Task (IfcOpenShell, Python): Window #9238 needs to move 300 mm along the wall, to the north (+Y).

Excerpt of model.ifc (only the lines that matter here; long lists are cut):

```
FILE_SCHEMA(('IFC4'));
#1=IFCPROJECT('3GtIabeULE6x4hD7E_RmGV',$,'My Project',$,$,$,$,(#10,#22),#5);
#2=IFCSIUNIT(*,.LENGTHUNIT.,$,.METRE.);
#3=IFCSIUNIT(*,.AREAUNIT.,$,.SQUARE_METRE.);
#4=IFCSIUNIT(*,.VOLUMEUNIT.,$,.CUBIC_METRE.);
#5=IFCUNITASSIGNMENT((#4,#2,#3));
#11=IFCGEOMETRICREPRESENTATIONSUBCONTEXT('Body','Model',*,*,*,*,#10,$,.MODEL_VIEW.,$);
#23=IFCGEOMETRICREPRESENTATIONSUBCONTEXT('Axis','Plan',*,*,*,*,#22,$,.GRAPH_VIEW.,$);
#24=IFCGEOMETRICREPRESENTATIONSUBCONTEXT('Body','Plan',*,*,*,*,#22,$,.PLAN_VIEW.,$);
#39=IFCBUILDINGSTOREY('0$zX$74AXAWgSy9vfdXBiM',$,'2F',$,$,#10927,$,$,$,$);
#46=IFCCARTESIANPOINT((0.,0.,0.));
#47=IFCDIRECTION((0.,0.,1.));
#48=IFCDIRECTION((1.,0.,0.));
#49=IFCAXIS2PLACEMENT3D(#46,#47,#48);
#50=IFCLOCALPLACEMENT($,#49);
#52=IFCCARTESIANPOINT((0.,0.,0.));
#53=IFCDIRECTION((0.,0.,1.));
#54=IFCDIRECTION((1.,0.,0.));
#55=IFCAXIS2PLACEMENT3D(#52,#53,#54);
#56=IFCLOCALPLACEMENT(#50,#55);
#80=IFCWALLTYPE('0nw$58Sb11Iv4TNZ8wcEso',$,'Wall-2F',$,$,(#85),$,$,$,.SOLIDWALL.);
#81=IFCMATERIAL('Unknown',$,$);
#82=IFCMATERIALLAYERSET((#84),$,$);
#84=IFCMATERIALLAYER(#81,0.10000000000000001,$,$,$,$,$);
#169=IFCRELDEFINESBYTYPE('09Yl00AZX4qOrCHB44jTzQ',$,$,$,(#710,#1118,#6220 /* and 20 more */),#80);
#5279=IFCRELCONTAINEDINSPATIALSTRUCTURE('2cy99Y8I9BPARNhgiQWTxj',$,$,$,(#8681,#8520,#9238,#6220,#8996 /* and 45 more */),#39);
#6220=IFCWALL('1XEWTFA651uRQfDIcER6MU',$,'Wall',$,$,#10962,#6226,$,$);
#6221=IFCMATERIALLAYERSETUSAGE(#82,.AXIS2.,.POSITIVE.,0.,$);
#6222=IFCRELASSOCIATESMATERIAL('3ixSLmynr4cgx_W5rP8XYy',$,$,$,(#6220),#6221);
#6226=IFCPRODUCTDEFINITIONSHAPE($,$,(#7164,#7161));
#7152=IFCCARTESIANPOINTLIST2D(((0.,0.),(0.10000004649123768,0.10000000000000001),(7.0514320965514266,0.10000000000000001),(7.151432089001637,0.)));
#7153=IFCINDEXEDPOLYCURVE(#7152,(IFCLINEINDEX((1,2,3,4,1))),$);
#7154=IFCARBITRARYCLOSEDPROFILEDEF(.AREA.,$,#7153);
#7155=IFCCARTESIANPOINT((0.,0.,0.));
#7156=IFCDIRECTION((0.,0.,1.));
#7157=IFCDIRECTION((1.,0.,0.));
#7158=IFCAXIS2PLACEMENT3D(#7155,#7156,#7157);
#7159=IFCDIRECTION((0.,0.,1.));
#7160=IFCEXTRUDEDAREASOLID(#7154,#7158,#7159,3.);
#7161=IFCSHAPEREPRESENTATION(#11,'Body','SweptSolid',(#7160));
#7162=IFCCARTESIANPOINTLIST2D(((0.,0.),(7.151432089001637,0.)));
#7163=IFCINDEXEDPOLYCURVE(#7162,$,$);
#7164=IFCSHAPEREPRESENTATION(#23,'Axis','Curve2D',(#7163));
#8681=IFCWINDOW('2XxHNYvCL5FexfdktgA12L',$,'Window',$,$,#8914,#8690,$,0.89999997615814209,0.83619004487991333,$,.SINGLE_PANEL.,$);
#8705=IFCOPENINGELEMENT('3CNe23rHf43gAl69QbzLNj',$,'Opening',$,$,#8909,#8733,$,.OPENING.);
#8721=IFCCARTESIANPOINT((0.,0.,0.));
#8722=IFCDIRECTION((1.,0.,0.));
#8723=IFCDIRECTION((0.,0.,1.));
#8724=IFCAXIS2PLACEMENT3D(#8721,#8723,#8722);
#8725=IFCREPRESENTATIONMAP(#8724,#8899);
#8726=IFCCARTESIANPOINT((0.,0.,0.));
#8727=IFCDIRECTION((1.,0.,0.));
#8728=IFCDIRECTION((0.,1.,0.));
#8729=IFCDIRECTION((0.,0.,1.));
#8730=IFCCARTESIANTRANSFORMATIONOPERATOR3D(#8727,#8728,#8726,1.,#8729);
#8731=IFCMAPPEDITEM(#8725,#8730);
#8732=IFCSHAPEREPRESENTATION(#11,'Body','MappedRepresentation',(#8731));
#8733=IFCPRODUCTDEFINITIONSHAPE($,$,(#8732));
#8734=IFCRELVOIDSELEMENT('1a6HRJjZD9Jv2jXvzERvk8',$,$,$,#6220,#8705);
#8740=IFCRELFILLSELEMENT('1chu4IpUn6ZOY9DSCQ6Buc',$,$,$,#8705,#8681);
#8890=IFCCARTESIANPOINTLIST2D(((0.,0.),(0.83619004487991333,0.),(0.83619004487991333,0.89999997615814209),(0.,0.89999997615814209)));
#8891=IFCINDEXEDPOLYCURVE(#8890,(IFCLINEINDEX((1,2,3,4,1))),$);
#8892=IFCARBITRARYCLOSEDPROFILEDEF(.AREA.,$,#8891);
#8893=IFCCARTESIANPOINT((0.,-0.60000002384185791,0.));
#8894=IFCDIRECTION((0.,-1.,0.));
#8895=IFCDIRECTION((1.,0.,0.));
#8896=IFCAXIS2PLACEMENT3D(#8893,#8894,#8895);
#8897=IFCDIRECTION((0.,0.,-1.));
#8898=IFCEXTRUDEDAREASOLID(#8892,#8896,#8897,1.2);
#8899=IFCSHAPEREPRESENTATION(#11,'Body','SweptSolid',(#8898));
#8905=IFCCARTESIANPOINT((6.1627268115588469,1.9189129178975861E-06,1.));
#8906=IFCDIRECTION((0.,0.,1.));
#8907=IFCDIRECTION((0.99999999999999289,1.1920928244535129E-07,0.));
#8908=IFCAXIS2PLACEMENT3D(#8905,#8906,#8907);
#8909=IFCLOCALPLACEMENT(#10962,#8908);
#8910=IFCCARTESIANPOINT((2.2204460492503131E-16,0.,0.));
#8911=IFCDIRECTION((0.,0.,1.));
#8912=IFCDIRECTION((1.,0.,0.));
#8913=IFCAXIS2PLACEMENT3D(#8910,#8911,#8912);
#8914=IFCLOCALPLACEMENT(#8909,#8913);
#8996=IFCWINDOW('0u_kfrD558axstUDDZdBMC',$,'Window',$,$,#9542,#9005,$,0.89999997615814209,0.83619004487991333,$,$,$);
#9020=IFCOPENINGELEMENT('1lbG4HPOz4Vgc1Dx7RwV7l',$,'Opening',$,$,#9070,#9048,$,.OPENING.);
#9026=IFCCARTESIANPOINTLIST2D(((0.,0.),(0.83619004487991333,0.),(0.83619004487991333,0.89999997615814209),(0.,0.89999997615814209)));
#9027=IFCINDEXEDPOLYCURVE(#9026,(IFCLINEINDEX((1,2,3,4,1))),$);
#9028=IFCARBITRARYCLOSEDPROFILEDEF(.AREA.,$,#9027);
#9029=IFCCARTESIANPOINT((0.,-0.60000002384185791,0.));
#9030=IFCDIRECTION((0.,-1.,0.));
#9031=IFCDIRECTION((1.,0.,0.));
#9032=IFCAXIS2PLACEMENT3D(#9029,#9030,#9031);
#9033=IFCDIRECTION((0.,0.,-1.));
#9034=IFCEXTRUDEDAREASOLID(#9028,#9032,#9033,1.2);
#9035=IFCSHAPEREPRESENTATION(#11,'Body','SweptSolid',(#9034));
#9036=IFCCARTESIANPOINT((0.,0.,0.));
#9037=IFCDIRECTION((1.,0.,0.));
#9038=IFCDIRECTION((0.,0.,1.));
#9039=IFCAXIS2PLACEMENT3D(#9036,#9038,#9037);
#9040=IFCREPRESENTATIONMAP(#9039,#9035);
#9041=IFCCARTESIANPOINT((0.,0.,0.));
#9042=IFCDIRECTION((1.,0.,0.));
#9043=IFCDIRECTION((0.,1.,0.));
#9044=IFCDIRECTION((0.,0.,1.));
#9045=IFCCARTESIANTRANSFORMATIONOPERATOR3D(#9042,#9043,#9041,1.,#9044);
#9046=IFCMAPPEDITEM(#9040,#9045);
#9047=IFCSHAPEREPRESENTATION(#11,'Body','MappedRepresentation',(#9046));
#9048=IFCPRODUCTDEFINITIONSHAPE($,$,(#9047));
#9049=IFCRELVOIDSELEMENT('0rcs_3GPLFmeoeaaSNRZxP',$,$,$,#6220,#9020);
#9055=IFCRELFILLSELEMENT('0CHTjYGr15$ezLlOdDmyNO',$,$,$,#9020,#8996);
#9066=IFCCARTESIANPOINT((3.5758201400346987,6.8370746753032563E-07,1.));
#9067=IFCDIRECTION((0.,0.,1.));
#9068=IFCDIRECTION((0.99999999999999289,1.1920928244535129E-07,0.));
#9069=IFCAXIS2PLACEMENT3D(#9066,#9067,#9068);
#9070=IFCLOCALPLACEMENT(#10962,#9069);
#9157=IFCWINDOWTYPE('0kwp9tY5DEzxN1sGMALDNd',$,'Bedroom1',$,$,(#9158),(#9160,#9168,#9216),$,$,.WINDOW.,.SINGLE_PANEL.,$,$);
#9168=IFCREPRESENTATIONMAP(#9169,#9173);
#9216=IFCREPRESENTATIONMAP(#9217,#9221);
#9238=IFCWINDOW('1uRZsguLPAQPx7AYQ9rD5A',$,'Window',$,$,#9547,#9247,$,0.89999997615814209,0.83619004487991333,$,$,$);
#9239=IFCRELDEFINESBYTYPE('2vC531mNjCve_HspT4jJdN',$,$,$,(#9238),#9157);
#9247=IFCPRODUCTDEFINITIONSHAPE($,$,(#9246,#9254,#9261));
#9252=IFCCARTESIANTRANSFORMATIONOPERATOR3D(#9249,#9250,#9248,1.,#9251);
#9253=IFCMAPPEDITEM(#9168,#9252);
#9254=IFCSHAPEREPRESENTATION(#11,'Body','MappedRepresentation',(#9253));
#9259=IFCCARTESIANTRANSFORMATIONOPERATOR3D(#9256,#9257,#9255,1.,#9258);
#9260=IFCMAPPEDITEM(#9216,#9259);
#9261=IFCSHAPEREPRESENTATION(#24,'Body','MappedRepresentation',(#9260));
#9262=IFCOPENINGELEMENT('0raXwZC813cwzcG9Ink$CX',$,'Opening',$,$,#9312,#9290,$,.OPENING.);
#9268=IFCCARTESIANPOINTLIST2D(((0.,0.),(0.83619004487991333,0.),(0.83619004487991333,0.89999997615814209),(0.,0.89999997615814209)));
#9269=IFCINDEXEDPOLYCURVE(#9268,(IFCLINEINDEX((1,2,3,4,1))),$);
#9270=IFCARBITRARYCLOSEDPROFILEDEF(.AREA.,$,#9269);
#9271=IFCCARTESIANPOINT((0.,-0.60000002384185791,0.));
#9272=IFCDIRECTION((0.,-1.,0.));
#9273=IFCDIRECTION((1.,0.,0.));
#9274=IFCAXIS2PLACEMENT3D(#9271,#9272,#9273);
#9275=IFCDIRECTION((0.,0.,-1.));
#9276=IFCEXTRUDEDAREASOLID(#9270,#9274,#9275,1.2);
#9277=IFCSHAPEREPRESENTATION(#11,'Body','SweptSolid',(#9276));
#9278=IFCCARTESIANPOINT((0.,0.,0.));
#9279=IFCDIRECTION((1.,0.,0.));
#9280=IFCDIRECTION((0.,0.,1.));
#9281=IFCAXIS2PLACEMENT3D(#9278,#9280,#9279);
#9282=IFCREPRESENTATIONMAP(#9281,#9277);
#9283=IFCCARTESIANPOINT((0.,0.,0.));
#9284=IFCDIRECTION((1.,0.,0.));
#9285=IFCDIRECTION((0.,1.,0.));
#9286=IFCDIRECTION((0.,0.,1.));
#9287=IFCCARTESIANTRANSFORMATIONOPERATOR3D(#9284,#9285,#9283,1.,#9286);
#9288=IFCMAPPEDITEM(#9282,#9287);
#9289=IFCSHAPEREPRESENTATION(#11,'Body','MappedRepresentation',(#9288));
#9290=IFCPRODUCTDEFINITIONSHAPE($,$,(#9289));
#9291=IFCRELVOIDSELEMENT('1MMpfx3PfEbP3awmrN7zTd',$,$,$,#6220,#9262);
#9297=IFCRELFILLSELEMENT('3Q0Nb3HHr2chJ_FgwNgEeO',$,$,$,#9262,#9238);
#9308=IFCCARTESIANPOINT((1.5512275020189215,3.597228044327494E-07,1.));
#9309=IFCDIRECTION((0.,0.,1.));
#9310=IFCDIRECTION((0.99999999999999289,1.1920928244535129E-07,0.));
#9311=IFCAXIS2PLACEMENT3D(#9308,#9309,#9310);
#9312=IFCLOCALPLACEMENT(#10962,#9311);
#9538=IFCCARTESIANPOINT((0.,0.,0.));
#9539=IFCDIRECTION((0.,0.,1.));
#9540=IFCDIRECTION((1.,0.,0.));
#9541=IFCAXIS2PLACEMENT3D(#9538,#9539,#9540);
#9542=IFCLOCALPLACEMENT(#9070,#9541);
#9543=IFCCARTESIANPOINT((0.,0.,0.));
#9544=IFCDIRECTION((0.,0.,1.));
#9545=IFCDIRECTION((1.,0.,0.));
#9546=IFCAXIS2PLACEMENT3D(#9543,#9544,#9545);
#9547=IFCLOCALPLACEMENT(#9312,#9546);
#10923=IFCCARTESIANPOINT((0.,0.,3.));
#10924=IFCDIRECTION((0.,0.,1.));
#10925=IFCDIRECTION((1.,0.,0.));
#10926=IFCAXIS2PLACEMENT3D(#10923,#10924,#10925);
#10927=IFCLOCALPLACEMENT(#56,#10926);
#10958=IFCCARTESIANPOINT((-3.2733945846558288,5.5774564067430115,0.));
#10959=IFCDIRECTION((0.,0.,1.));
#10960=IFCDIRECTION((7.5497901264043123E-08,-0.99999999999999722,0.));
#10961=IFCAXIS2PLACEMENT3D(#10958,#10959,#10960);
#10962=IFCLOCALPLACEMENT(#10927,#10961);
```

```python
import ifcopenshell
import ifcopenshell.api.geometry
import ifcopenshell.util.placement
import ifcopenshell.util.unit

model = ifcopenshell.open("model.ifc")
unit_scale = ifcopenshell.util.unit.calculate_unit_scale(model)

window = model.by_guid("1uRZsguLPAQPx7AYQ9rD5A")
opening = window.FillsVoids[0].RelatingOpeningElement
wall = opening.VoidsElements[0].RelatingBuildingElement

wall_matrix = ifcopenshell.util.placement.get_local_placement(wall.ObjectPlacement)
shift = wall_matrix[:3, 0] * -0.3 / unit_scale
before = ifcopenshell.util.placement.get_local_placement(window.ObjectPlacement)[:3, 3].copy()

# The window is placed relative to its opening, so it follows when the opening moves.
matrix = ifcopenshell.util.placement.get_local_placement(opening.ObjectPlacement)
matrix[:3, 3] += shift
ifcopenshell.api.geometry.edit_object_placement(
    model, product=opening, matrix=matrix, is_si=False, should_transform_children=True
)

after = ifcopenshell.util.placement.get_local_placement(window.ObjectPlacement)[:3, 3]
print("window moved by", (after - before).round(3) + 0.0)

model.write("model_rev.ifc")
```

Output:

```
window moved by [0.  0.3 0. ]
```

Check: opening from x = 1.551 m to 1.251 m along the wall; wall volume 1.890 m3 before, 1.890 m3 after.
